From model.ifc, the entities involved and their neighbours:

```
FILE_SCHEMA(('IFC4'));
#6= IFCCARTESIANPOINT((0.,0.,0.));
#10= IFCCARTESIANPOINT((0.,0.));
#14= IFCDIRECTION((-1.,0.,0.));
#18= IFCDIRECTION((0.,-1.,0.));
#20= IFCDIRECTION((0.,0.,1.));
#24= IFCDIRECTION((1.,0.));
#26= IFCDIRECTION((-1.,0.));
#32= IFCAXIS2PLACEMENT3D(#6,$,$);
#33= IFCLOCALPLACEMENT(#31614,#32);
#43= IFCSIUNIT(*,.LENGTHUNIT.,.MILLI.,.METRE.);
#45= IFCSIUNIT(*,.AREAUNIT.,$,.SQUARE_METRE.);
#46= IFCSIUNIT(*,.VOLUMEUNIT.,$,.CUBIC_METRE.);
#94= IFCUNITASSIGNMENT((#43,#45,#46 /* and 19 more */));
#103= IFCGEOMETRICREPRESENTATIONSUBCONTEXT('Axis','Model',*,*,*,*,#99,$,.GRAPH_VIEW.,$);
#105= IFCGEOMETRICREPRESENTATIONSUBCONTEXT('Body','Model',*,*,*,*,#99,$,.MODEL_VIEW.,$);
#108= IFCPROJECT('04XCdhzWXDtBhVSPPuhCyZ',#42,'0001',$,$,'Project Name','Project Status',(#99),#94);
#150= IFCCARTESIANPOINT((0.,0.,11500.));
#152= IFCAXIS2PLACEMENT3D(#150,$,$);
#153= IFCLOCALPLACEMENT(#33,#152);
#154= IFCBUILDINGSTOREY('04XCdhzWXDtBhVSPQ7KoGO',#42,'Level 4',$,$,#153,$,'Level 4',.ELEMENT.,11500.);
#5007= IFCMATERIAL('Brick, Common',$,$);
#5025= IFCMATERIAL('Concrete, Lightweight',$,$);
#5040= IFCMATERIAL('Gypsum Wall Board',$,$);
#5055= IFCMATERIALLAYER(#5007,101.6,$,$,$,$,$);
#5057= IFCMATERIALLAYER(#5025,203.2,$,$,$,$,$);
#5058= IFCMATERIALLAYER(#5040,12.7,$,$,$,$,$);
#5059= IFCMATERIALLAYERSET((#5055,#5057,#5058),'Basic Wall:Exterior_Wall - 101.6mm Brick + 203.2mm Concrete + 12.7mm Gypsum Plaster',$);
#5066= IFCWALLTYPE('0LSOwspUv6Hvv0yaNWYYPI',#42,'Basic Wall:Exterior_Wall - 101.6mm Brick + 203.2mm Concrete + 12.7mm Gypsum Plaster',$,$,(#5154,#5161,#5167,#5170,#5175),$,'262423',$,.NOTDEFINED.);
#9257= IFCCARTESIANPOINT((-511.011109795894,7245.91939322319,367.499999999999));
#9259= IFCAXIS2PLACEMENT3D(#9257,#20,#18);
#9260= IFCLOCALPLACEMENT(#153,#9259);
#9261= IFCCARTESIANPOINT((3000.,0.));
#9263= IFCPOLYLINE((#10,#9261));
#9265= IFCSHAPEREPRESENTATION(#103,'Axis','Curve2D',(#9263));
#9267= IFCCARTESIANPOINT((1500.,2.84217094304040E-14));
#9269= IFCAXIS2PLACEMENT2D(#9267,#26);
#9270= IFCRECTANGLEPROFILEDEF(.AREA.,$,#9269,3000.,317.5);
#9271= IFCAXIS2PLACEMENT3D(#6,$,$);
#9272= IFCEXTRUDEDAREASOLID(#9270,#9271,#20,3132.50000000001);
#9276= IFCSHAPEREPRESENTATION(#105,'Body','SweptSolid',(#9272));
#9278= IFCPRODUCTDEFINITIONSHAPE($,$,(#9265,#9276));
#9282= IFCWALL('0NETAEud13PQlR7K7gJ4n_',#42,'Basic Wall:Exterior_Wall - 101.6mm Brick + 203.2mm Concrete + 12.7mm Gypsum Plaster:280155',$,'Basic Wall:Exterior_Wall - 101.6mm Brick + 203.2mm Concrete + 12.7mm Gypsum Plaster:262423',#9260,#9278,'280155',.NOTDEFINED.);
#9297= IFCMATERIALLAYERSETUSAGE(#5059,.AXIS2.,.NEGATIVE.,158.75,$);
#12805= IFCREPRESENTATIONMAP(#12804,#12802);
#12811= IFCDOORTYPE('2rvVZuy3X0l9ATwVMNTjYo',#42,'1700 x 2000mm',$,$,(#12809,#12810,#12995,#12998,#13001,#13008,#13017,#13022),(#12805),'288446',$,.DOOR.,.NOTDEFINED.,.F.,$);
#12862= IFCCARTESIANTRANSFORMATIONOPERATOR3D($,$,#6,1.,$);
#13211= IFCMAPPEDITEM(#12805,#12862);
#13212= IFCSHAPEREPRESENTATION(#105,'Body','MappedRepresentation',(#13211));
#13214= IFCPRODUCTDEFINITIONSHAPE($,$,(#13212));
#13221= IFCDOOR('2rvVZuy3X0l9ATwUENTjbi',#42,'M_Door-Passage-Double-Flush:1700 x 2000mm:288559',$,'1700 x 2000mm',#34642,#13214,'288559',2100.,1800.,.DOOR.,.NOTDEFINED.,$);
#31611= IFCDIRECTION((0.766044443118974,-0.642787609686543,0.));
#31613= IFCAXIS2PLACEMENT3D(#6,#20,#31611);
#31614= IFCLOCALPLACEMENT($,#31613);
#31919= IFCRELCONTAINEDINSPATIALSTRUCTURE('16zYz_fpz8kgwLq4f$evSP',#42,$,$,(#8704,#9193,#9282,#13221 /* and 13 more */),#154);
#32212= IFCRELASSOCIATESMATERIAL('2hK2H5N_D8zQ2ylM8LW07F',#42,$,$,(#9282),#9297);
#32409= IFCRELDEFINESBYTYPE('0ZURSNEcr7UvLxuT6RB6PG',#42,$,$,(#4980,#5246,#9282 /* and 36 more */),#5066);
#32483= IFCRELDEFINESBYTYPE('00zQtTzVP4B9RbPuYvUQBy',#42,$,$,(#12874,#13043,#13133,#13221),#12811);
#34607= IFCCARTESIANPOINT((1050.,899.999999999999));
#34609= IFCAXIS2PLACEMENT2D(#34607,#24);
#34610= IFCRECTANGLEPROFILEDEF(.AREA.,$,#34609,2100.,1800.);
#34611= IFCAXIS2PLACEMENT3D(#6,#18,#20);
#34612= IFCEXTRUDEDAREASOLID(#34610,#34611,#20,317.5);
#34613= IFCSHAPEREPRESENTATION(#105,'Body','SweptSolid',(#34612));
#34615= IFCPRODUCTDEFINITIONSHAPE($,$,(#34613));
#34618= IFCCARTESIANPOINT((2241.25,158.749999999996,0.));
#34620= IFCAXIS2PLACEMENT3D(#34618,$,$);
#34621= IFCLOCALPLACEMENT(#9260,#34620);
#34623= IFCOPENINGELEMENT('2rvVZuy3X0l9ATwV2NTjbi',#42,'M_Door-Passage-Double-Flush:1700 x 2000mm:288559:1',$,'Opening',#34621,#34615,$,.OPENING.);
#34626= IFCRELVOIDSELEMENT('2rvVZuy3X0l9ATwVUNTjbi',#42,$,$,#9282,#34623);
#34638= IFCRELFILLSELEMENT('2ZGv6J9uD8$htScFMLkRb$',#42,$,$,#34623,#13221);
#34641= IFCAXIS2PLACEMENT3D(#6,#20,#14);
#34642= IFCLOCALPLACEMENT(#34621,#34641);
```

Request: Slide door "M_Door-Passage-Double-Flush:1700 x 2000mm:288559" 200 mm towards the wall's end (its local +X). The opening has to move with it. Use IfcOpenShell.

```python
import ifcopenshell
import ifcopenshell.api.geometry
import ifcopenshell.util.placement

model = ifcopenshell.open("model.ifc")

door = model.by_guid("2rvVZuy3X0l9ATwUENTjbi")
opening = door.FillsVoids[0].RelatingOpeningElement
wall = opening.VoidsElements[0].RelatingBuildingElement

wall_matrix = ifcopenshell.util.placement.get_local_placement(wall.ObjectPlacement)
shift = wall_matrix[:3, 0] * 200.0
before = ifcopenshell.util.placement.get_local_placement(door.ObjectPlacement)[:3, 3].copy()

# The door is placed relative to its opening, so it follows when the opening moves.
matrix = ifcopenshell.util.placement.get_local_placement(opening.ObjectPlacement)
matrix[:3, 3] += shift
ifcopenshell.api.geometry.edit_object_placement(
    model, product=opening, matrix=matrix, is_si=False, should_transform_children=True
)

after = ifcopenshell.util.placement.get_local_placement(door.ObjectPlacement)[:3, 3]
print("door moved by", (after - before).round(3) + 0.0)

model.write("model_rev.ifc")
```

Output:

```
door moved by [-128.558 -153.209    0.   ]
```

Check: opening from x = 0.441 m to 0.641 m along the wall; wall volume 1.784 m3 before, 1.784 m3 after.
